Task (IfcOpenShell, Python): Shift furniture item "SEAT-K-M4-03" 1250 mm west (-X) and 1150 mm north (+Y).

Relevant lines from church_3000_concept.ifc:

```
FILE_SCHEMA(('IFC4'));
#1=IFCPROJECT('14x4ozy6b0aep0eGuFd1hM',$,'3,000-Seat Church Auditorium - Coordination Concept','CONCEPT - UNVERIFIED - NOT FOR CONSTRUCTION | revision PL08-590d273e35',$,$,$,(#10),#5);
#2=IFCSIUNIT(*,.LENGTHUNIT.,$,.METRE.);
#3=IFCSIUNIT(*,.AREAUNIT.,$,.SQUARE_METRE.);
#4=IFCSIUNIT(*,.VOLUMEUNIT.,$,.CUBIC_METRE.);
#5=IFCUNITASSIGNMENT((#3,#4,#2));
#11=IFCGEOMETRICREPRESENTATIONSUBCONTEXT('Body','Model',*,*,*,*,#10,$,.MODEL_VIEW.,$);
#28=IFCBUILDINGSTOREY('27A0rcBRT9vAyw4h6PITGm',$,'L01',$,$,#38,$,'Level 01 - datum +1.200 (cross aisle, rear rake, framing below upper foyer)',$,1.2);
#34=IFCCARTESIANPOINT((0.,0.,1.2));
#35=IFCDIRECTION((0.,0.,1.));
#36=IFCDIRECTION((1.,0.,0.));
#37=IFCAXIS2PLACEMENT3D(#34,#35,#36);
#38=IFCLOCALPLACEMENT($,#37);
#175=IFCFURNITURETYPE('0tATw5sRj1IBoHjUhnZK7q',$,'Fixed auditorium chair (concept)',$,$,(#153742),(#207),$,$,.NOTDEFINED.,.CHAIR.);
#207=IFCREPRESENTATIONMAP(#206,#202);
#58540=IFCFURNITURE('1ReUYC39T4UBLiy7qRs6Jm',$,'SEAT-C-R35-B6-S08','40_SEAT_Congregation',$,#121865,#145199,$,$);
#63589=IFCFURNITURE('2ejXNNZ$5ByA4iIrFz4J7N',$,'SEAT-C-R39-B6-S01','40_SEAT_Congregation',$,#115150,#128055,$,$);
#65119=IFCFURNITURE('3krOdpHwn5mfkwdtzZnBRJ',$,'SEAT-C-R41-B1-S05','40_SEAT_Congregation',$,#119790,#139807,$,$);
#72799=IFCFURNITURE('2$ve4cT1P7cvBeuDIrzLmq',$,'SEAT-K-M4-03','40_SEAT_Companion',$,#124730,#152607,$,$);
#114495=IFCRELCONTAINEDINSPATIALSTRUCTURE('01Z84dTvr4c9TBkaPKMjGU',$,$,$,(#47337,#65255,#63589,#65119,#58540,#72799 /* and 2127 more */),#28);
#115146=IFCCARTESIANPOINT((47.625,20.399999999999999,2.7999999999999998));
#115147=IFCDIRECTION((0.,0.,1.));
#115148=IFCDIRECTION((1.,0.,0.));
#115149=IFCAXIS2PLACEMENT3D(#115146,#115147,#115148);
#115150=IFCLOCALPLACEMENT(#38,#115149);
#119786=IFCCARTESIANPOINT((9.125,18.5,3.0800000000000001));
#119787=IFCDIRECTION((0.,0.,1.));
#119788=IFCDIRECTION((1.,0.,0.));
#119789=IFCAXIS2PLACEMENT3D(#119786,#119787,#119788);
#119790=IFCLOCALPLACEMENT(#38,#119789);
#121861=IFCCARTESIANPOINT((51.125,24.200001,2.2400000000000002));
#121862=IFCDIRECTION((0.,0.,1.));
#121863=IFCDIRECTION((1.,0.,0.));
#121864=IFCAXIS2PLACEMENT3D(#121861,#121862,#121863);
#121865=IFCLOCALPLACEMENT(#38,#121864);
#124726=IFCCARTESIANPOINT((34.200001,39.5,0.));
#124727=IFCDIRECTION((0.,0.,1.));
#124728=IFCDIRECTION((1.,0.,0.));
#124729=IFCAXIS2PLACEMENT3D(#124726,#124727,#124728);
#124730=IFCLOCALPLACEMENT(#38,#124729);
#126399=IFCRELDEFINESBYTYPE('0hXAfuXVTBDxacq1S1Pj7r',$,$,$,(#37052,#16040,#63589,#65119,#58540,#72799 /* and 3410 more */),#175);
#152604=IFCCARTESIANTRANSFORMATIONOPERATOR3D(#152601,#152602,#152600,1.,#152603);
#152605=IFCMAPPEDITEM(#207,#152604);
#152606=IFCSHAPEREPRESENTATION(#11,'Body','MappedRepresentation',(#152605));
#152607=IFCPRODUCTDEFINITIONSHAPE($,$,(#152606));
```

```python
import ifcopenshell
import ifcopenshell.api.geometry
import ifcopenshell.util.placement
import ifcopenshell.util.unit

model = ifcopenshell.open("church_3000_concept.ifc")
unit_scale = ifcopenshell.util.unit.calculate_unit_scale(model)

item = model.by_id(72799)
matrix = ifcopenshell.util.placement.get_local_placement(item.ObjectPlacement)
matrix[0, 3] -= 1.25 / unit_scale
matrix[1, 3] += 1.15 / unit_scale
ifcopenshell.api.geometry.edit_object_placement(model, product=item, matrix=matrix, is_si=False)

print(ifcopenshell.util.placement.get_local_placement(item.ObjectPlacement).round(3) + 0.0)

model.write("church_3000_concept_v2.ifc")
```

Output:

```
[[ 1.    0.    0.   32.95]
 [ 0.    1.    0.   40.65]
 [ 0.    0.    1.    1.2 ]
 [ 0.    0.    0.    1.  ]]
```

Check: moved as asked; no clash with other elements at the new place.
